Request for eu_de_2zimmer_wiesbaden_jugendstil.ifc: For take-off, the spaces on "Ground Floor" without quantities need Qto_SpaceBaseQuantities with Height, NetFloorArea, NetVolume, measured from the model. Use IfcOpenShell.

First a look at what the model holds.

```python
import ifcopenshell
import ifcopenshell.util.element
import ifcopenshell.util.unit

model = ifcopenshell.open("eu_de_2zimmer_wiesbaden_jugendstil.ifc")
print(model.schema)
for unit_type in ("LENGTHUNIT", "AREAUNIT", "VOLUMEUNIT"):
    print(unit_type, ifcopenshell.util.unit.calculate_unit_scale(model, unit_type))
storey = next(s for s in model.by_type("IfcBuildingStorey") if s.Name == "Ground Floor")
spaces = [e for e in ifcopenshell.util.element.get_decomposition(storey) if e.is_a("IfcSpace")]
for e in sorted(spaces, key=lambda e: e.id()):
    print(e.id(), e.is_a(), e.Name, list(ifcopenshell.util.element.get_psets(e, qtos_only=True)), sep=" | ")
```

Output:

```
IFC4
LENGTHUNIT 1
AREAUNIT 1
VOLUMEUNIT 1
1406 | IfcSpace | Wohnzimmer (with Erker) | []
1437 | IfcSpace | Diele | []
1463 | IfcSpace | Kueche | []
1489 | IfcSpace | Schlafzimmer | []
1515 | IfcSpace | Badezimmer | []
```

```python
import ifcopenshell
import ifcopenshell.api.pset
import ifcopenshell.geom
import ifcopenshell.util.element
import ifcopenshell.util.shape
import ifcopenshell.util.unit

model = ifcopenshell.open("eu_de_2zimmer_wiesbaden_jugendstil.ifc")
unit_scale = ifcopenshell.util.unit.calculate_unit_scale(model)
area_scale = ifcopenshell.util.unit.calculate_unit_scale(model, "AREAUNIT")
volume_scale = ifcopenshell.util.unit.calculate_unit_scale(model, "VOLUMEUNIT")
settings = ifcopenshell.geom.settings()

storey = next(s for s in model.by_type("IfcBuildingStorey") if s.Name == "Ground Floor")
spaces = [e for e in ifcopenshell.util.element.get_decomposition(storey) if e.is_a("IfcSpace")]

for e in sorted(spaces, key=lambda e: e.id()):
    if ifcopenshell.util.element.get_psets(e, qtos_only=True, should_inherit=False):
        continue
    # Geometry comes back in metres, in the element's own axes.
    shape = ifcopenshell.geom.create_shape(settings, e)
    values = {
        "Height": ifcopenshell.util.shape.get_z(shape.geometry) / unit_scale,
        "NetFloorArea": ifcopenshell.util.shape.get_footprint_area(shape.geometry) / area_scale,
        "NetVolume": ifcopenshell.util.shape.get_volume(shape.geometry) / volume_scale,
    }
    qto = ifcopenshell.api.pset.add_qto(model, product=e, name="Qto_SpaceBaseQuantities")
    ifcopenshell.api.pset.edit_qto(model, qto=qto, properties=values)
    print(e.id(), {k: round(v, 3) for k, v in values.items()})

model.write("eu_de_2zimmer_wiesbaden_jugendstil-out.ifc")
```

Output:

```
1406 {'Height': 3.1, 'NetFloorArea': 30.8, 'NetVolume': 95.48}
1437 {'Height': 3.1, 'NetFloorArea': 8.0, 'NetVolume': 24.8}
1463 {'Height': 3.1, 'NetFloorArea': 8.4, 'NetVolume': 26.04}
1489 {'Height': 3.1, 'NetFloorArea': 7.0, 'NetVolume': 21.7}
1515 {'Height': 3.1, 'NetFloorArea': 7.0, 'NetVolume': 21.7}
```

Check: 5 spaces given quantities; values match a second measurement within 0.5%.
